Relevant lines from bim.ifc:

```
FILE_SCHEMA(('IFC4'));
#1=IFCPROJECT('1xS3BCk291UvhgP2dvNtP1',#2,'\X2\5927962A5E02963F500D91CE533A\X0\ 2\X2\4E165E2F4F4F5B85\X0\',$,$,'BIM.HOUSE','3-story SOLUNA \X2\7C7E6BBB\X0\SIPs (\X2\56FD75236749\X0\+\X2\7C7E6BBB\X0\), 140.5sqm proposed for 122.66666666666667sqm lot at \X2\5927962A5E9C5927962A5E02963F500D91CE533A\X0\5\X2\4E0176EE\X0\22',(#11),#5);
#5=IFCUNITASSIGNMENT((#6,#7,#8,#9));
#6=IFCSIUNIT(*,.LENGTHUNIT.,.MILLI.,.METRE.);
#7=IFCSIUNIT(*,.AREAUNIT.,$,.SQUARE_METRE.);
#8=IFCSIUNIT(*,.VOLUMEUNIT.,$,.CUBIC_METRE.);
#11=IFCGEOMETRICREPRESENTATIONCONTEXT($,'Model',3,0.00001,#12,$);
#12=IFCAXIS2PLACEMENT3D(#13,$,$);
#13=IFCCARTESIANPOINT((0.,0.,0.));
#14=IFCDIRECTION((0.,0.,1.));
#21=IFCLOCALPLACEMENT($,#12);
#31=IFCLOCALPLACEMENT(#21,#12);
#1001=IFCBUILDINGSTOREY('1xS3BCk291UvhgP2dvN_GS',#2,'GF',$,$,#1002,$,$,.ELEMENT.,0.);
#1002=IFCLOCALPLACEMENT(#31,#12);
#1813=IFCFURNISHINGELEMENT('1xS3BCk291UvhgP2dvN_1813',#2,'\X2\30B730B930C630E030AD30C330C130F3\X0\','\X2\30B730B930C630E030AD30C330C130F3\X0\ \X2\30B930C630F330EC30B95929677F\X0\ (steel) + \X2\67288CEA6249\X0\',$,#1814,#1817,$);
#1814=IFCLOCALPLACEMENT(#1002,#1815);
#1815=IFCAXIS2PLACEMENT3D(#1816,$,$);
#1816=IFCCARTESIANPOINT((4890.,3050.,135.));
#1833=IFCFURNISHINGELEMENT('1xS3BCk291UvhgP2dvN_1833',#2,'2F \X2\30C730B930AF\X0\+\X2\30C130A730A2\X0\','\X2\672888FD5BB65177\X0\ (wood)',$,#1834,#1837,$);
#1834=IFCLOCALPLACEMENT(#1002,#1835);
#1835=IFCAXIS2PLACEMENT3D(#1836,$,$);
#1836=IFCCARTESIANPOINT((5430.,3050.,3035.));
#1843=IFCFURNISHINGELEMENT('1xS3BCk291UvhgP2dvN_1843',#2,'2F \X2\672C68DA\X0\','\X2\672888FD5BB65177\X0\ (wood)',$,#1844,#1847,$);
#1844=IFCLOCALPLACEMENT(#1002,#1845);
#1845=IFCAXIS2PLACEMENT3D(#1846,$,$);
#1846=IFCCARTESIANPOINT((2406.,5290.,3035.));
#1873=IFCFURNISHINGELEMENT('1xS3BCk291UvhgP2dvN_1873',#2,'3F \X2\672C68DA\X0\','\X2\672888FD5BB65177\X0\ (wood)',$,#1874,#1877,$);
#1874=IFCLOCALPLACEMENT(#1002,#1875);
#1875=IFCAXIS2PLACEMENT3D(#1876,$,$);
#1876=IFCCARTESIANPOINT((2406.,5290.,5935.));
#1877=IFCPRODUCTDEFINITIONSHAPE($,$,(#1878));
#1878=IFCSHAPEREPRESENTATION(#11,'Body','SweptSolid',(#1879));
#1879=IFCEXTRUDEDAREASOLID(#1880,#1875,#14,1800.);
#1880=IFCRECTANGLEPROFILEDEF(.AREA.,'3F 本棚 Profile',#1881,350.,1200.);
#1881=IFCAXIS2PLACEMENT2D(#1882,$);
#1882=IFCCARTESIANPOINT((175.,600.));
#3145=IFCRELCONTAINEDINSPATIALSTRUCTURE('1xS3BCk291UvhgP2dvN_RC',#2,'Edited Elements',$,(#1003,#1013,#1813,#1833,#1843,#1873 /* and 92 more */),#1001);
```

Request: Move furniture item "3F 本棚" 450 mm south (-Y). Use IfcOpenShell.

```python
import ifcopenshell
import ifcopenshell.api.geometry
import ifcopenshell.util.placement
import ifcopenshell.util.unit

model = ifcopenshell.open("bim.ifc")
unit_scale = ifcopenshell.util.unit.calculate_unit_scale(model)

item = model.by_guid("1xS3BCk291UvhgP2dvN_1873")
matrix = ifcopenshell.util.placement.get_local_placement(item.ObjectPlacement)
matrix[1, 3] -= 0.45 / unit_scale
ifcopenshell.api.geometry.edit_object_placement(model, product=item, matrix=matrix, is_si=False)

print(ifcopenshell.util.placement.get_local_placement(item.ObjectPlacement).round(3) + 0.0)

model.write("bim_v2.ifc")
```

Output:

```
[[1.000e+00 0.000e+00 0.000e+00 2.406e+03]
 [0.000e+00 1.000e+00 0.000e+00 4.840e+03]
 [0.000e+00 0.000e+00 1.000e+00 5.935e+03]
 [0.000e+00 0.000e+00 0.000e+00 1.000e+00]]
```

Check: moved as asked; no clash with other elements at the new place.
